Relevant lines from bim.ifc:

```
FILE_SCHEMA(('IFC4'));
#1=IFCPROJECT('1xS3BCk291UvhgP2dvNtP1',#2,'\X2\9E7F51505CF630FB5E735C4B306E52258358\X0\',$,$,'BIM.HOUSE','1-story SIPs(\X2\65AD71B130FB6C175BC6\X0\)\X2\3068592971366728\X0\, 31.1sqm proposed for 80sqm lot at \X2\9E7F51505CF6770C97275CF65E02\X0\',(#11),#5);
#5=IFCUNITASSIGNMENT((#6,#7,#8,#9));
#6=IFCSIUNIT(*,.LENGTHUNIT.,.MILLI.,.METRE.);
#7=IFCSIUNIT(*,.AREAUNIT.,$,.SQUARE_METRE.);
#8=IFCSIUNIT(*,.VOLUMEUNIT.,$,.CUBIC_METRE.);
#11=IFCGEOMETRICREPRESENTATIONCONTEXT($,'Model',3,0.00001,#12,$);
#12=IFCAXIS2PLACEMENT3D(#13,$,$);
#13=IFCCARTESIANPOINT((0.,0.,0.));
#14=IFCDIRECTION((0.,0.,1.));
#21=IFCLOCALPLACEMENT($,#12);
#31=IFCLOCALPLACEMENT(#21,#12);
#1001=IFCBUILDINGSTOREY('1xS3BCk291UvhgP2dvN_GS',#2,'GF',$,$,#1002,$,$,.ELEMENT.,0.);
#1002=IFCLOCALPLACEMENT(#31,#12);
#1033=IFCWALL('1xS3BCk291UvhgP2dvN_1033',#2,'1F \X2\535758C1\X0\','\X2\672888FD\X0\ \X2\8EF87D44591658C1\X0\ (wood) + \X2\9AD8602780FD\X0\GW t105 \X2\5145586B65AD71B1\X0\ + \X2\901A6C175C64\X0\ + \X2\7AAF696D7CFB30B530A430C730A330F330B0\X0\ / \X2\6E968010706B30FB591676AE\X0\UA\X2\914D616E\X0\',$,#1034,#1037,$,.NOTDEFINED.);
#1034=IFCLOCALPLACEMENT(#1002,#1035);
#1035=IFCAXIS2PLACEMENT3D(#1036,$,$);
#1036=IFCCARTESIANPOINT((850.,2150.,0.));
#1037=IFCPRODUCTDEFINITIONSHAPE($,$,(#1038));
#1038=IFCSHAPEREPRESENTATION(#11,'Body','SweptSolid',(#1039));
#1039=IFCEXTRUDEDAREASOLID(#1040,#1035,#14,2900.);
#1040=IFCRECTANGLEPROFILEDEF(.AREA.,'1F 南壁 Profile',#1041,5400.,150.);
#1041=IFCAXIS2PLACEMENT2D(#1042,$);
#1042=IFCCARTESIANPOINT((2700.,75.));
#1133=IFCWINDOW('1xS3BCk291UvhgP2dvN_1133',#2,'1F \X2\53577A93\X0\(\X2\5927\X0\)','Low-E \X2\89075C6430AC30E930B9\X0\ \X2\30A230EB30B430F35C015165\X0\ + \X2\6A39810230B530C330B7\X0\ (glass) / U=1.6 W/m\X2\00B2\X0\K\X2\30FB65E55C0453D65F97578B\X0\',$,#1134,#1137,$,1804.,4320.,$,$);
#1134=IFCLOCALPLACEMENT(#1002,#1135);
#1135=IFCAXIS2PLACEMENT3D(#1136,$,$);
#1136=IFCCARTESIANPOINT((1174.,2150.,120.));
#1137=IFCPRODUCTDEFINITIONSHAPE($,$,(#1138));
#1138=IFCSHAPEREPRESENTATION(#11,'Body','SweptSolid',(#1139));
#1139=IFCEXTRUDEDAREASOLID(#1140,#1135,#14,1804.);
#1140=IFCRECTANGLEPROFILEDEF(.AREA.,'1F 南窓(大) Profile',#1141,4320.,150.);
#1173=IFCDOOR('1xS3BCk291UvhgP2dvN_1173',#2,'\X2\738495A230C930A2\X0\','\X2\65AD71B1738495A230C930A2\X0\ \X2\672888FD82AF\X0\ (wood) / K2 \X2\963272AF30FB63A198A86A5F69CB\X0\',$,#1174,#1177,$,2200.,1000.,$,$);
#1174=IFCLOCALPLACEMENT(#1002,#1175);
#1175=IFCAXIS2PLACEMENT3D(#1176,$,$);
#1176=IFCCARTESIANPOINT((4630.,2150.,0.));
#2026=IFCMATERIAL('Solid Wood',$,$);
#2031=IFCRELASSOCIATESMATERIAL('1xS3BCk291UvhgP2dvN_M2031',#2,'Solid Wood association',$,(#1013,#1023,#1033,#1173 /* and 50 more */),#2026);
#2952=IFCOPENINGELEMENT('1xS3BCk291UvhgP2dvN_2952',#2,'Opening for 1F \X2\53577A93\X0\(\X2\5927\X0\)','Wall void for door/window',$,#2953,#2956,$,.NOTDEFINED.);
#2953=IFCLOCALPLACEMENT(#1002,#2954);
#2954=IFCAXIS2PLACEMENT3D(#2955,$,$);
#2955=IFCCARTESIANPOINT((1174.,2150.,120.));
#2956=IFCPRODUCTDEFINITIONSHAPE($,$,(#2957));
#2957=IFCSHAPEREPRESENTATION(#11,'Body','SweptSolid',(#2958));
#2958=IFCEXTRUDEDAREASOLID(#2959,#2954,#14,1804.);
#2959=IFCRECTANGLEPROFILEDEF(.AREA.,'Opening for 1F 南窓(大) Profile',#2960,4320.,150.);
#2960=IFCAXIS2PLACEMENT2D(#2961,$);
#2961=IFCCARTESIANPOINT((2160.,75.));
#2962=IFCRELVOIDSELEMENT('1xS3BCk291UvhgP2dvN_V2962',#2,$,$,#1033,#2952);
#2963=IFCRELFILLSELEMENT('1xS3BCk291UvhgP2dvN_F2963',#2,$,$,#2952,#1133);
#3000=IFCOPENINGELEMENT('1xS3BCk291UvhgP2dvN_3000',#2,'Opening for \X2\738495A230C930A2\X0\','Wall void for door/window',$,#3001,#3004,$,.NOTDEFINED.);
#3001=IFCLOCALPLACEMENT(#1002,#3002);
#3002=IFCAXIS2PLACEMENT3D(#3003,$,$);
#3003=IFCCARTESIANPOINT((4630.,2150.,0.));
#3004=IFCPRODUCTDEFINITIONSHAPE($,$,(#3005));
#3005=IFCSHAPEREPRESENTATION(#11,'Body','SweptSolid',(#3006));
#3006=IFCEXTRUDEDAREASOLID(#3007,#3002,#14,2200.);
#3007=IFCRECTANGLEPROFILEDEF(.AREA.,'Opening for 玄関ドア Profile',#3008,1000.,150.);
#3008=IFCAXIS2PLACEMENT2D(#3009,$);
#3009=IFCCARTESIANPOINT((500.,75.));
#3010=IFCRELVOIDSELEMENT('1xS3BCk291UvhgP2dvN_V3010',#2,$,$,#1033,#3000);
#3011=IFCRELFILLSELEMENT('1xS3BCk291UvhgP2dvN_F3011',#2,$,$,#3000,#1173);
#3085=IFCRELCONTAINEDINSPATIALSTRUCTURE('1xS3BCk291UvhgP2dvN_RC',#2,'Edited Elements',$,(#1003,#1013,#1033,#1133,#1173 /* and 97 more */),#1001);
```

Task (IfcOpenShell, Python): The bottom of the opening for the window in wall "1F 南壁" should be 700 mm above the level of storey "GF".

```python
import numpy as np
import ifcopenshell
import ifcopenshell.api.geometry
import ifcopenshell.geom
import ifcopenshell.util.element
import ifcopenshell.util.placement
import ifcopenshell.util.shape
import ifcopenshell.util.unit

model = ifcopenshell.open("bim.ifc")
unit_scale = ifcopenshell.util.unit.calculate_unit_scale(model)

window = model.by_guid("1xS3BCk291UvhgP2dvN_1133")
opening = window.FillsVoids[0].RelatingOpeningElement
storey = ifcopenshell.util.element.get_container(window, ifc_class="IfcBuildingStorey")
level = ifcopenshell.util.placement.get_local_placement(storey.ObjectPlacement)[2, 3]

# The opening's origin need not be at the sill, so measure its lowest point.
shape = ifcopenshell.geom.create_shape(ifcopenshell.geom.settings(), opening)
bottom = ifcopenshell.util.shape.get_shape_bottom_elevation(shape, shape.geometry) / unit_scale
dz = level + 0.7 / unit_scale - bottom

shift = np.array([0.0, 0.0, dz])
# The window is not placed relative to its opening, so move both.
for product in (opening, window):
    matrix = ifcopenshell.util.placement.get_local_placement(product.ObjectPlacement)
    matrix[:3, 3] += shift
    ifcopenshell.api.geometry.edit_object_placement(model, product=product, matrix=matrix, is_si=False)

print(f"moved by {dz * unit_scale:+.3f} m")

model.write("bim_edited.ifc")
```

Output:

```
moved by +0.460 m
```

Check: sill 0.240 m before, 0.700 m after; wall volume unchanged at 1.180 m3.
